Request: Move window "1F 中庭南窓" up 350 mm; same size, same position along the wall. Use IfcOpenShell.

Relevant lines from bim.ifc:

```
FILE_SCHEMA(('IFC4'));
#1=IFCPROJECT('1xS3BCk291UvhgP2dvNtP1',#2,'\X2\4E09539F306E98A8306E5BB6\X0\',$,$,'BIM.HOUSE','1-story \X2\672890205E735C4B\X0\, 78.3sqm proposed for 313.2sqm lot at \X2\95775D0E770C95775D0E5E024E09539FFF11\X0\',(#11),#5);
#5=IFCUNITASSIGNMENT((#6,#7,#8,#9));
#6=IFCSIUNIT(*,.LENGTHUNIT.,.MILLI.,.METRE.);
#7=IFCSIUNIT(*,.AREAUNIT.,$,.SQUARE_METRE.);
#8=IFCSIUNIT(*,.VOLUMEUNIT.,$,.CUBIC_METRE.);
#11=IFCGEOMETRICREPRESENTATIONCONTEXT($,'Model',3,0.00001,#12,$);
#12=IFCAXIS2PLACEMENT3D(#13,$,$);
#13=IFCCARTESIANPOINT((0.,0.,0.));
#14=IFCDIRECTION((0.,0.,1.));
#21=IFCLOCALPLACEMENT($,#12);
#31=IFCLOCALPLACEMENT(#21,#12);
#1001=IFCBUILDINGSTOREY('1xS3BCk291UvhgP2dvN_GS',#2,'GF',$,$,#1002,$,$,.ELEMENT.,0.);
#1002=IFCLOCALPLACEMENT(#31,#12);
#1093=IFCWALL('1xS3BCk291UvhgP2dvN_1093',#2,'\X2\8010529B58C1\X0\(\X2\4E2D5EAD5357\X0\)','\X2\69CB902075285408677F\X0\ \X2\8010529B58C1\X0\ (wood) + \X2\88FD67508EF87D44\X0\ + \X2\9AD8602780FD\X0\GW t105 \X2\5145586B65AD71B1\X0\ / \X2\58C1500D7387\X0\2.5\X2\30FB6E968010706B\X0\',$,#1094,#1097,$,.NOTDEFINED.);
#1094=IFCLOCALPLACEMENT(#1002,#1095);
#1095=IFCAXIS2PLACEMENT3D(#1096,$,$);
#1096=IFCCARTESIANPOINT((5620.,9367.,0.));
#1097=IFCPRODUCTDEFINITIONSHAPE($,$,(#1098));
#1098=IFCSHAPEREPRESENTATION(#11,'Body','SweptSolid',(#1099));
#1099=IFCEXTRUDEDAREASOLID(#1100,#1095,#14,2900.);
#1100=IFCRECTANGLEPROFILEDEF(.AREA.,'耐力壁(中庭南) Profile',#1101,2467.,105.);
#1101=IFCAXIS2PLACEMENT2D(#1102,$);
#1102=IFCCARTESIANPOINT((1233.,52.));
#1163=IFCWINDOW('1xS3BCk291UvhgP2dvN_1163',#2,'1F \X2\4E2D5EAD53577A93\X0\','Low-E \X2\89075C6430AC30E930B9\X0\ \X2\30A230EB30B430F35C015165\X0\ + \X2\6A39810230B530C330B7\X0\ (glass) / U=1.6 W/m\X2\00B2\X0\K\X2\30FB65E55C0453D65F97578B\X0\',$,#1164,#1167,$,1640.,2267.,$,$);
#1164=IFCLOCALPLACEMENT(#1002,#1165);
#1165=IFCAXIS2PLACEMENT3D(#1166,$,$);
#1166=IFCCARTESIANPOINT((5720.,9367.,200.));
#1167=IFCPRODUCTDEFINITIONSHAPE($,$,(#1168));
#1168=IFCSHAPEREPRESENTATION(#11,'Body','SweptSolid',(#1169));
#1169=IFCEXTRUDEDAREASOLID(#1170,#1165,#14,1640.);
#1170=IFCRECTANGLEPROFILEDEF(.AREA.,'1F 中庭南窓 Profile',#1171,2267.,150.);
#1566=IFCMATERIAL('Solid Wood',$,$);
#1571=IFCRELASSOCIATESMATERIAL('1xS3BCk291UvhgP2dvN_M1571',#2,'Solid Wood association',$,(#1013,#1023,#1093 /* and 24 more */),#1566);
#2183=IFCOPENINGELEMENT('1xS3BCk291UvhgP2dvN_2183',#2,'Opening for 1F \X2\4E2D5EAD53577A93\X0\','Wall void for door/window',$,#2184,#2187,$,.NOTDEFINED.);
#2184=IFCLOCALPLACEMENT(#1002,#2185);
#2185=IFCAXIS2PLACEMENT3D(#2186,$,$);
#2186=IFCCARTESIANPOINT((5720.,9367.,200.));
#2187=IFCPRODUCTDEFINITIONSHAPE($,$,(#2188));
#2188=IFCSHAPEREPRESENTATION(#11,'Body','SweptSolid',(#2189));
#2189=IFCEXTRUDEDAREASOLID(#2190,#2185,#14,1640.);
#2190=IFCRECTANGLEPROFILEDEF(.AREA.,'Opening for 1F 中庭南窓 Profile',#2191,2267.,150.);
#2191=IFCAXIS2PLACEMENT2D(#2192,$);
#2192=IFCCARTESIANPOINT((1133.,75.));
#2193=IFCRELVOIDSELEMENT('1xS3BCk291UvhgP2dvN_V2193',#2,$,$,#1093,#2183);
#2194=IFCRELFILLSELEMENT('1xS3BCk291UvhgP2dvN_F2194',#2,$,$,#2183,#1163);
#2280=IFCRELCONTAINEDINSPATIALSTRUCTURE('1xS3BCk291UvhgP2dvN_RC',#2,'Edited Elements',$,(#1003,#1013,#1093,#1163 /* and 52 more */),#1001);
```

```python
import numpy as np
import ifcopenshell
import ifcopenshell.api.geometry
import ifcopenshell.util.placement
import ifcopenshell.util.unit

model = ifcopenshell.open("bim.ifc")
unit_scale = ifcopenshell.util.unit.calculate_unit_scale(model)

window = model.by_guid("1xS3BCk291UvhgP2dvN_1163")
opening = window.FillsVoids[0].RelatingOpeningElement
dz = 350.0

shift = np.array([0.0, 0.0, dz])
# The window is not placed relative to its opening, so move both.
for product in (opening, window):
    matrix = ifcopenshell.util.placement.get_local_placement(product.ObjectPlacement)
    matrix[:3, 3] += shift
    ifcopenshell.api.geometry.edit_object_placement(model, product=product, matrix=matrix, is_si=False)

print(f"moved by {dz * unit_scale:+.3f} m")

model.write("bim_rev.ifc")
```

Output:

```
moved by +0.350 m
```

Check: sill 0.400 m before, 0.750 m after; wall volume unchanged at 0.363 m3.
